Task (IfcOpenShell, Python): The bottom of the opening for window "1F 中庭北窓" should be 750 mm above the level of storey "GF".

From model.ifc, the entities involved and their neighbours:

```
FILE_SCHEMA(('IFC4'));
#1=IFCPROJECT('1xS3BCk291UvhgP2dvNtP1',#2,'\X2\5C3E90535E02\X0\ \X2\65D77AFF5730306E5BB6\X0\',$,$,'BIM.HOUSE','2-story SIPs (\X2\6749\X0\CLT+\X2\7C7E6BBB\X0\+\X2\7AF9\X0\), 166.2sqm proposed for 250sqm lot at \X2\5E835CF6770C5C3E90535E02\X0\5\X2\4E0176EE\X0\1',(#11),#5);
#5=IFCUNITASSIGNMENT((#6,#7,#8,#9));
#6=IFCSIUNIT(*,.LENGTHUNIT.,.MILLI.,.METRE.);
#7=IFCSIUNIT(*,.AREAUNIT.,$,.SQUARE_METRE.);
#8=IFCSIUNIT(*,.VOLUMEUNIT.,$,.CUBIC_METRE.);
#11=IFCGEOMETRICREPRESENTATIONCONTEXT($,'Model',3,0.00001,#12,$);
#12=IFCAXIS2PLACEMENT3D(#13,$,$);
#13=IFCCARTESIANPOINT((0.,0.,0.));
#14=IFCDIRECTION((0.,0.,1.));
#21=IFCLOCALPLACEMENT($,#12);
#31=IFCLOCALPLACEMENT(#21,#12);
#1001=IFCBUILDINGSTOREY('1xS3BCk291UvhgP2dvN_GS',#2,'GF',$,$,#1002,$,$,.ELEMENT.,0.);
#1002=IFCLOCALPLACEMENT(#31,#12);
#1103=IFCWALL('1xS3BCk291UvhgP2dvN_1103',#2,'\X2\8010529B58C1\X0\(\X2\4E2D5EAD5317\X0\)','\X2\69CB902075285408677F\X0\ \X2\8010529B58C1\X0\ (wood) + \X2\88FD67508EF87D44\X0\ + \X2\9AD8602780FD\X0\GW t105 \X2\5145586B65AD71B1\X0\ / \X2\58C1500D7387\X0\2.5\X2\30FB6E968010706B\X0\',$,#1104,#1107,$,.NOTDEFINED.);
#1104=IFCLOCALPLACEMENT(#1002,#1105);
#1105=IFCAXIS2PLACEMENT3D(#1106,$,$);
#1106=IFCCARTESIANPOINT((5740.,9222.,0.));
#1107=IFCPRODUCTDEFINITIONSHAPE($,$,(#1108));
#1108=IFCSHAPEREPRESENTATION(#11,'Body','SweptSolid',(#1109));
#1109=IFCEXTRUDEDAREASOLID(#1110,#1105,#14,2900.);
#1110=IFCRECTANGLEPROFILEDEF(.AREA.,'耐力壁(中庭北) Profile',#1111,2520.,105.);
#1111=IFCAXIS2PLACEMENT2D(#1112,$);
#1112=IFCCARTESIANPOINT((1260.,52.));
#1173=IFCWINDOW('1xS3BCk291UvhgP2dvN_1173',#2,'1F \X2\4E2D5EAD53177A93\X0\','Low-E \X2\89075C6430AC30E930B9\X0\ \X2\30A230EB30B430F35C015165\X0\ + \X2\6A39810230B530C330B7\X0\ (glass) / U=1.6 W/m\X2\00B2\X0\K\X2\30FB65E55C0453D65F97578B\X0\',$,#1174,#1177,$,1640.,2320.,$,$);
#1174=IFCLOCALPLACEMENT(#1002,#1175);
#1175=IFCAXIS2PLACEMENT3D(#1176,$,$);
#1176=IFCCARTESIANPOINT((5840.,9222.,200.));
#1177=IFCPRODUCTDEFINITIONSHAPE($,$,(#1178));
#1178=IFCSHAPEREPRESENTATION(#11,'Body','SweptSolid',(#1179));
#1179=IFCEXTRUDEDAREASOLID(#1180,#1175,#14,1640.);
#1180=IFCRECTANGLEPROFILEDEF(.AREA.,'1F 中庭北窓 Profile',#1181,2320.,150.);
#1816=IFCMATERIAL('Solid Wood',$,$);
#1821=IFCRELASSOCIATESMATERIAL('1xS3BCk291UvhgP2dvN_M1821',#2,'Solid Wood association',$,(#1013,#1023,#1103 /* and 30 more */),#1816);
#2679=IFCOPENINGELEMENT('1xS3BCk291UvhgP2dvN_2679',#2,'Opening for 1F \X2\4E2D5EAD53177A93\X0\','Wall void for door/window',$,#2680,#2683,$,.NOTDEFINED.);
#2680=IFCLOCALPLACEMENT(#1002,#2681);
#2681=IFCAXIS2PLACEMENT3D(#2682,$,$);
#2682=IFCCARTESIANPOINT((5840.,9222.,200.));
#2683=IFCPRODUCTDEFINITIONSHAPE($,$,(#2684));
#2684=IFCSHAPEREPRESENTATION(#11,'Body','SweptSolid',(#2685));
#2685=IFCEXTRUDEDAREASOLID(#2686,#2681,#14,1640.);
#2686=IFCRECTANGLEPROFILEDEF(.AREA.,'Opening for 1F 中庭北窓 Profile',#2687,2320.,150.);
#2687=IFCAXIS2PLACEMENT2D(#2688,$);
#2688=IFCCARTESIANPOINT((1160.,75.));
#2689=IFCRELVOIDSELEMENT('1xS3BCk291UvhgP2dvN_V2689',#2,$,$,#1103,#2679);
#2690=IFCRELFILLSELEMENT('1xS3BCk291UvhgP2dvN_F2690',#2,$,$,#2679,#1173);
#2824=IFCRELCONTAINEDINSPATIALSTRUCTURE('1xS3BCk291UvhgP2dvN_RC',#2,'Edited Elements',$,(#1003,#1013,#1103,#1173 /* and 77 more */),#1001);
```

```python
import numpy as np
import ifcopenshell
import ifcopenshell.api.geometry
import ifcopenshell.geom
import ifcopenshell.util.element
import ifcopenshell.util.placement
import ifcopenshell.util.shape
import ifcopenshell.util.unit

model = ifcopenshell.open("model.ifc")
unit_scale = ifcopenshell.util.unit.calculate_unit_scale(model)

window = model.by_id(1173)
opening = window.FillsVoids[0].RelatingOpeningElement
storey = ifcopenshell.util.element.get_container(window, ifc_class="IfcBuildingStorey")
level = ifcopenshell.util.placement.get_local_placement(storey.ObjectPlacement)[2, 3]

# The opening's origin need not be at the sill, so measure its lowest point.
shape = ifcopenshell.geom.create_shape(ifcopenshell.geom.settings(), opening)
bottom = ifcopenshell.util.shape.get_shape_bottom_elevation(shape, shape.geometry) / unit_scale
dz = level + 750.0 - bottom

shift = np.array([0.0, 0.0, dz])
# The window is not placed relative to its opening, so move both.
for product in (opening, window):
    matrix = ifcopenshell.util.placement.get_local_placement(product.ObjectPlacement)
    matrix[:3, 3] += shift
    ifcopenshell.api.geometry.edit_object_placement(model, product=product, matrix=matrix, is_si=False)

print(f"moved by {dz * unit_scale:+.3f} m")

model.write("model_v2.ifc")
```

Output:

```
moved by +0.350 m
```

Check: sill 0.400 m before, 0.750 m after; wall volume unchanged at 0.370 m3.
